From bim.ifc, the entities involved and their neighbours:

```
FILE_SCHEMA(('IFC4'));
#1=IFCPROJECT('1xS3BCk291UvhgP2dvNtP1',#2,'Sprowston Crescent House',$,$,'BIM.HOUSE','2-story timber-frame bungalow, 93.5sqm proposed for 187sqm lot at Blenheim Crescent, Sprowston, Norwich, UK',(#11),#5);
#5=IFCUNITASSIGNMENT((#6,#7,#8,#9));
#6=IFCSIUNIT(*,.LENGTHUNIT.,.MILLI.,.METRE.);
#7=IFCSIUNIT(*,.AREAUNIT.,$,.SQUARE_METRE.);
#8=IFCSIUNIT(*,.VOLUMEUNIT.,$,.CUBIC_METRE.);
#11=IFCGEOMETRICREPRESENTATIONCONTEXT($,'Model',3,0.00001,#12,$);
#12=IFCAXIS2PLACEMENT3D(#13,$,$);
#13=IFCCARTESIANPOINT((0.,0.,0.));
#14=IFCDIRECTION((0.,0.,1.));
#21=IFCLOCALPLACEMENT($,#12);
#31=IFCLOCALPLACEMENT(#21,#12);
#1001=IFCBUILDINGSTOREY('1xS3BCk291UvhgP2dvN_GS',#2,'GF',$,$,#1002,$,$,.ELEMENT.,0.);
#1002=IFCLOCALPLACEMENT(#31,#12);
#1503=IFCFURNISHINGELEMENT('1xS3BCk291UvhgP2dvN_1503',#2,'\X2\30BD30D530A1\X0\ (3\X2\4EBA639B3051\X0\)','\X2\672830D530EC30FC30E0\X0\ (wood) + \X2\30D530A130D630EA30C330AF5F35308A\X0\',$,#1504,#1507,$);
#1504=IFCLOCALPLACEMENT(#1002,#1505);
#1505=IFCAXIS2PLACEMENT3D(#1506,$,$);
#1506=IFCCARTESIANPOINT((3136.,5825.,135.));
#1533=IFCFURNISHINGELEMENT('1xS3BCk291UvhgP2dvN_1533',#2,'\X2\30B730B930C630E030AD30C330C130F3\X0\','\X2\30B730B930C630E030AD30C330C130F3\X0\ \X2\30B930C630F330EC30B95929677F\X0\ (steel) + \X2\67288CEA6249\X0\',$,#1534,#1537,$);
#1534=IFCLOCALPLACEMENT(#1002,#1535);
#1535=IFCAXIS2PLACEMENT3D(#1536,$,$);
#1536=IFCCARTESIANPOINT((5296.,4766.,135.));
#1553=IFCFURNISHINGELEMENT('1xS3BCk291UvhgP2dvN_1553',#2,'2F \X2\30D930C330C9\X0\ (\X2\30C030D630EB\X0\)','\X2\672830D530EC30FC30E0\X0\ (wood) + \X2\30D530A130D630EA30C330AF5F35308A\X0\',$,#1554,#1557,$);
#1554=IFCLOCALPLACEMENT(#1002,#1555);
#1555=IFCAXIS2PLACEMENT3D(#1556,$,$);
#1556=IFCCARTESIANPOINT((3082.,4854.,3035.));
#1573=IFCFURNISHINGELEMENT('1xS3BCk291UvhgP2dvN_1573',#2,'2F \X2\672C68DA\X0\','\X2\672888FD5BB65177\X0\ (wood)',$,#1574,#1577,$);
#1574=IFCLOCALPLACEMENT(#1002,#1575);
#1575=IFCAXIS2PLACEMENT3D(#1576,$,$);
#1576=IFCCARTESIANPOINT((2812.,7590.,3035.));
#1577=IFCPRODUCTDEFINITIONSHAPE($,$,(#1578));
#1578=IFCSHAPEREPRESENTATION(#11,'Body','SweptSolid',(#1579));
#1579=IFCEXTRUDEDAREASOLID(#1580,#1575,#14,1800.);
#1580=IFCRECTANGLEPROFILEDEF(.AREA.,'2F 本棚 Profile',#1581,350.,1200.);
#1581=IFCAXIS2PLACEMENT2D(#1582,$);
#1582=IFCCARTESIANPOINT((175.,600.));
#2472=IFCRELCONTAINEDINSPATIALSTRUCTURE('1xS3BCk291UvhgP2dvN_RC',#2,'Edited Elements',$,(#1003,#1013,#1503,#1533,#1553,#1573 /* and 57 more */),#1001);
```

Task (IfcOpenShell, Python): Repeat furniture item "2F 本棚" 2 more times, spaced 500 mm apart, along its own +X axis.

```python
import ifcopenshell
import ifcopenshell.api.geometry
import ifcopenshell.api.root
import ifcopenshell.util.element
import ifcopenshell.util.placement

model = ifcopenshell.open("bim.ifc")


def reuse_history(source, copy):
    """copy_class also copies each property set's owner history, people and application; keep the originals."""
    for rel in copy.IsDefinedBy:
        if rel.is_a("IfcRelDefinesByProperties") and (history := rel.RelatingPropertyDefinition.OwnerHistory):
            rel.RelatingPropertyDefinition.OwnerHistory = source.OwnerHistory
            ifcopenshell.util.element.remove_deep2(model, history)


source = model.by_id(1573)
base = ifcopenshell.util.placement.get_local_placement(source.ObjectPlacement)
step = base[:3, 0] * 500.0

for i in range(1, 3):
    copy = ifcopenshell.api.root.copy_class(model, product=source)
    copy.Representation = ifcopenshell.util.element.copy_deep(
        model, source.Representation, exclude=["IfcGeometricRepresentationContext", "IfcRepresentationMap"]
    )
    reuse_history(source, copy)
    matrix = base.copy()
    matrix[:3, 3] += i * step
    print("added at", matrix[:3, 3].round(3) + 0.0)
    ifcopenshell.api.geometry.edit_object_placement(model, product=copy, matrix=matrix, is_si=False)

model.write("bim_v2.ifc")
```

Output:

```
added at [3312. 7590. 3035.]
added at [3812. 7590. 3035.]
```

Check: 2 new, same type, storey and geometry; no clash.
